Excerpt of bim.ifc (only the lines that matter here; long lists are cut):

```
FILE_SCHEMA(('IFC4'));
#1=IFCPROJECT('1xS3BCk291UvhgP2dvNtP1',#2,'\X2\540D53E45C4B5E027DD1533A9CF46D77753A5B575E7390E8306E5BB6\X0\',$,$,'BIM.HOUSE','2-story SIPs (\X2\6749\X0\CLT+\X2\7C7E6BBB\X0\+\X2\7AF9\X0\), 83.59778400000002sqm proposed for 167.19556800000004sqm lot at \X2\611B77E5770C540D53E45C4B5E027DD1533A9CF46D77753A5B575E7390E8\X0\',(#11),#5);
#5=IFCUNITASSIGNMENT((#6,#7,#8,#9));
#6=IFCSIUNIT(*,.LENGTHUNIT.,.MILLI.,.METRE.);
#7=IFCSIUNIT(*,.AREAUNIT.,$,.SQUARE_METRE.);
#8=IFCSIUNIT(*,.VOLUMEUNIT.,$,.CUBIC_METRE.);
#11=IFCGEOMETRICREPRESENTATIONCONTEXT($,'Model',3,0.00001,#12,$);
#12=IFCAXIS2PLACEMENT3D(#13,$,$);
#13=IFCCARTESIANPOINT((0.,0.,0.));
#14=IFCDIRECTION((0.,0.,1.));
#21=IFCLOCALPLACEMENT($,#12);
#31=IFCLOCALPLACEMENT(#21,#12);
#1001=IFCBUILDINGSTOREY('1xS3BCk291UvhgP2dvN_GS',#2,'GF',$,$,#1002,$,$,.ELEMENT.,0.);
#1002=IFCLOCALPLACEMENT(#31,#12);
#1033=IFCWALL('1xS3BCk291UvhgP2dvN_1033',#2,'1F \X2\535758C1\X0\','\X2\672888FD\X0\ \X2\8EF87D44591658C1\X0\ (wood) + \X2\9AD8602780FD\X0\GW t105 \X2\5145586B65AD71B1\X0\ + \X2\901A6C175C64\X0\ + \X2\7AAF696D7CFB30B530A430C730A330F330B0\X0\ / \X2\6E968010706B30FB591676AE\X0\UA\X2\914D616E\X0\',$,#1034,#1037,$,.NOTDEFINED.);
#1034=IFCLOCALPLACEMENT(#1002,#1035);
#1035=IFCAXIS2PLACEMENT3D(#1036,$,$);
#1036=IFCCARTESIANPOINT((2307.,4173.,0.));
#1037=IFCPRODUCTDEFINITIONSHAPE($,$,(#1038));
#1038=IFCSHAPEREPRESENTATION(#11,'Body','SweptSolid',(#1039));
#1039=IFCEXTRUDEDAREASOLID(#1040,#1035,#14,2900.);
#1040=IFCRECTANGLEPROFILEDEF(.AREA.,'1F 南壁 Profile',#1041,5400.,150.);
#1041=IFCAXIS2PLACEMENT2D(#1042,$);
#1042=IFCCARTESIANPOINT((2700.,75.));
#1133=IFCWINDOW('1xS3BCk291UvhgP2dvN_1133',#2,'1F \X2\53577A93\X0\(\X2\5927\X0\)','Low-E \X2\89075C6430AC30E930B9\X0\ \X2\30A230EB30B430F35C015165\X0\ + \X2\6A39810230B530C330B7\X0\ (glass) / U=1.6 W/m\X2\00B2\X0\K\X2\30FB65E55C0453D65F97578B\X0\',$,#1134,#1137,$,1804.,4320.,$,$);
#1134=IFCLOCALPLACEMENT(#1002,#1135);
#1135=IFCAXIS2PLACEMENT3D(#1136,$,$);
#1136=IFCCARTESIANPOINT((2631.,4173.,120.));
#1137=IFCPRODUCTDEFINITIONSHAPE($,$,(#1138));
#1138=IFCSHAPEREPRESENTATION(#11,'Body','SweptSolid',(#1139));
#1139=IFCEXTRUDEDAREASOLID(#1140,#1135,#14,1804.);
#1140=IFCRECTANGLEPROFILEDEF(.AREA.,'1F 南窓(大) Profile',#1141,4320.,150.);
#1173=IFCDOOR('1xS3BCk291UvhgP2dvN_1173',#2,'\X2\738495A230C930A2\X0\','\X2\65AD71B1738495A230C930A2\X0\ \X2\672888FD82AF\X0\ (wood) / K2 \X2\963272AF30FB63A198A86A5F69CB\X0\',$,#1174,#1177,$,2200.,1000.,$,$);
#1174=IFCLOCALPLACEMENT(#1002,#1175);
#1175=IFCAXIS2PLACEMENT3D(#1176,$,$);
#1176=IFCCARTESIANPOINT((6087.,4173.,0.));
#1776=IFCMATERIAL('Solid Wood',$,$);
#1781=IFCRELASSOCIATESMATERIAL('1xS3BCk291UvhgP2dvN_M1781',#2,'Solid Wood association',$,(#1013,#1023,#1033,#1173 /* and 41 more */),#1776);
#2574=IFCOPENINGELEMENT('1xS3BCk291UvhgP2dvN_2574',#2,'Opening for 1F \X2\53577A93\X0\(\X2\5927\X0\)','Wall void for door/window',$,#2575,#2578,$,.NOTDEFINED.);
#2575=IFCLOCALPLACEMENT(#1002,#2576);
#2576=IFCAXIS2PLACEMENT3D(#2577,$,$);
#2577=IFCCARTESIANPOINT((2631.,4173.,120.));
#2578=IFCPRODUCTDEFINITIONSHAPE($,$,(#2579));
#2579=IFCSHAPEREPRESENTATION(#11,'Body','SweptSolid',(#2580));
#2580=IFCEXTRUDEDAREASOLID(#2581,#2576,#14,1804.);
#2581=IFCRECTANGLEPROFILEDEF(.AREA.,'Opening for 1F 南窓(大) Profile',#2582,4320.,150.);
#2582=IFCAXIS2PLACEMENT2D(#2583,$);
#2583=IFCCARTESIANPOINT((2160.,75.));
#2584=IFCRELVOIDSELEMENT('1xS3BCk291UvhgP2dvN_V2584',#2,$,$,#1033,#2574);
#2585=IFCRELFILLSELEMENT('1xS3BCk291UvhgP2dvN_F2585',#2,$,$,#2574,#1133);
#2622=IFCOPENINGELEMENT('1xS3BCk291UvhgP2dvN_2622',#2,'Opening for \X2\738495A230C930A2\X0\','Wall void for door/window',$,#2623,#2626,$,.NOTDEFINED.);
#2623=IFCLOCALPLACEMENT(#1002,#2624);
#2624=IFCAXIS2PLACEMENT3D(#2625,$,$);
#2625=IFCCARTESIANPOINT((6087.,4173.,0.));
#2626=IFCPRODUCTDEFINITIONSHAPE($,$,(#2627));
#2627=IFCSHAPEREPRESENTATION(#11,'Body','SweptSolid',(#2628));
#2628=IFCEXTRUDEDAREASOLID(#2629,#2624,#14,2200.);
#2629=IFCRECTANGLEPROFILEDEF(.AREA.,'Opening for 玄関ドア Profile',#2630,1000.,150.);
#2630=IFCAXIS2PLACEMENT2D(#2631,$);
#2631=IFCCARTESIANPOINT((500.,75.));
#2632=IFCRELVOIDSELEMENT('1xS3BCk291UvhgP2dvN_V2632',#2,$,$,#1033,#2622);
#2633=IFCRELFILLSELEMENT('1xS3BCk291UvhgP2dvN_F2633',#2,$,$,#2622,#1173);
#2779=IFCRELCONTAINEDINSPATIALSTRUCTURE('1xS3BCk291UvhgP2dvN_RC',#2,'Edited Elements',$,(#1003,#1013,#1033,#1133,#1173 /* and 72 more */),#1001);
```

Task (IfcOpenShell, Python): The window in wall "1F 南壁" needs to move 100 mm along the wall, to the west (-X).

```python
import ifcopenshell
import ifcopenshell.api.geometry
import ifcopenshell.util.placement

model = ifcopenshell.open("bim.ifc")

window = model.by_guid("1xS3BCk291UvhgP2dvN_1133")
opening = window.FillsVoids[0].RelatingOpeningElement
wall = opening.VoidsElements[0].RelatingBuildingElement

wall_matrix = ifcopenshell.util.placement.get_local_placement(wall.ObjectPlacement)
shift = wall_matrix[:3, 0] * -100.0
before = ifcopenshell.util.placement.get_local_placement(window.ObjectPlacement)[:3, 3].copy()

# The window is not placed relative to its opening, so move both.
for product in (opening, window):
    matrix = ifcopenshell.util.placement.get_local_placement(product.ObjectPlacement)
    matrix[:3, 3] += shift
    ifcopenshell.api.geometry.edit_object_placement(model, product=product, matrix=matrix, is_si=False)

after = ifcopenshell.util.placement.get_local_placement(window.ObjectPlacement)[:3, 3]
print("window moved by", (after - before).round(3) + 0.0)

model.write("bim_updated.ifc")
```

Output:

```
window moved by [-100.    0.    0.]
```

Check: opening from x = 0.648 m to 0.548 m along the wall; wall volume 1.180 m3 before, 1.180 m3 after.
